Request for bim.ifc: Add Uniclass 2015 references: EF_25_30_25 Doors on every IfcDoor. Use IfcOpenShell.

First a look at what the model holds.

```python
import ifcopenshell

model = ifcopenshell.open("bim.ifc")
print(model.schema)
print("classifications:", [c.Name for c in model.by_type("IfcClassification")])
for ifc_class in ("IfcDoor", "IfcRoof", "IfcStair", "IfcWall", "IfcWindow"):
    print(ifc_class, len(model.by_type(ifc_class)))
```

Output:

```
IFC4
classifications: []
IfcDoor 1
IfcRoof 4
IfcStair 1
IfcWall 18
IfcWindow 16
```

```python
import ifcopenshell
import ifcopenshell.api.classification

model = ifcopenshell.open("bim.ifc")

system = ifcopenshell.api.classification.add_classification(model, classification="Uniclass 2015")

codes = {
    "IfcDoor": ("EF_25_30_25", "Doors"),
}
for ifc_class, (code, name) in codes.items():
    products = model.by_type(ifc_class)
    ifcopenshell.api.classification.add_reference(
        model, products=products, classification=system, identification=code, name=name
    )
    print(code, len(products))

model.write("bim_updated.ifc")
```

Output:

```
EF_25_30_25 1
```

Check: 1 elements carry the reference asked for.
